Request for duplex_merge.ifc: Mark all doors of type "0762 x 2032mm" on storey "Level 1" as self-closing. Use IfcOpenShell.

First a look at what the model holds.

```python
import ifcopenshell
import ifcopenshell.util.element

model = ifcopenshell.open("duplex_merge.ifc")
print(model.schema)
storey = next(s for s in model.by_type("IfcBuildingStorey") if s.Name == "Level 1")
doors = [e for e in ifcopenshell.util.element.get_decomposition(storey) if e.is_a("IfcDoor")]
seen = {}
for e in doors:
    element_type = ifcopenshell.util.element.get_type(e)
    key = (element_type.Name if element_type != e and element_type else None, ifcopenshell.util.element.get_pset(e, "Pset_DoorCommon", "SelfClosing"))
    seen[key] = seen.get(key, 0) + 1
for (name, value), count in sorted(seen.items(), key=str):
    print(count, "x", name, "|", value)
```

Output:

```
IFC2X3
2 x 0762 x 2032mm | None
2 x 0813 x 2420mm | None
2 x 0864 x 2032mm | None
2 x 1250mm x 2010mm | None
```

```python
import ifcopenshell
import ifcopenshell.api.pset
import ifcopenshell.util.element

model = ifcopenshell.open("duplex_merge.ifc")

storey = next(s for s in model.by_type("IfcBuildingStorey") if s.Name == "Level 1")
doors = [e for e in ifcopenshell.util.element.get_decomposition(storey) if e.is_a("IfcDoor")]

count = 0
for e in doors:
    element_type = ifcopenshell.util.element.get_type(e)
    if element_type in (None, e) or element_type.Name != "0762 x 2032mm":
        continue
    # add_pset returns the element's existing set when there is one.
    pset = ifcopenshell.api.pset.add_pset(model, product=e, name="Pset_DoorCommon")
    ifcopenshell.api.pset.edit_pset(model, pset=pset, properties={"SelfClosing": True})
    count += 1

print(count, "doors updated")

model.write("duplex_merge_updated.ifc")
```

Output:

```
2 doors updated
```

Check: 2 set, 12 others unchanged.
